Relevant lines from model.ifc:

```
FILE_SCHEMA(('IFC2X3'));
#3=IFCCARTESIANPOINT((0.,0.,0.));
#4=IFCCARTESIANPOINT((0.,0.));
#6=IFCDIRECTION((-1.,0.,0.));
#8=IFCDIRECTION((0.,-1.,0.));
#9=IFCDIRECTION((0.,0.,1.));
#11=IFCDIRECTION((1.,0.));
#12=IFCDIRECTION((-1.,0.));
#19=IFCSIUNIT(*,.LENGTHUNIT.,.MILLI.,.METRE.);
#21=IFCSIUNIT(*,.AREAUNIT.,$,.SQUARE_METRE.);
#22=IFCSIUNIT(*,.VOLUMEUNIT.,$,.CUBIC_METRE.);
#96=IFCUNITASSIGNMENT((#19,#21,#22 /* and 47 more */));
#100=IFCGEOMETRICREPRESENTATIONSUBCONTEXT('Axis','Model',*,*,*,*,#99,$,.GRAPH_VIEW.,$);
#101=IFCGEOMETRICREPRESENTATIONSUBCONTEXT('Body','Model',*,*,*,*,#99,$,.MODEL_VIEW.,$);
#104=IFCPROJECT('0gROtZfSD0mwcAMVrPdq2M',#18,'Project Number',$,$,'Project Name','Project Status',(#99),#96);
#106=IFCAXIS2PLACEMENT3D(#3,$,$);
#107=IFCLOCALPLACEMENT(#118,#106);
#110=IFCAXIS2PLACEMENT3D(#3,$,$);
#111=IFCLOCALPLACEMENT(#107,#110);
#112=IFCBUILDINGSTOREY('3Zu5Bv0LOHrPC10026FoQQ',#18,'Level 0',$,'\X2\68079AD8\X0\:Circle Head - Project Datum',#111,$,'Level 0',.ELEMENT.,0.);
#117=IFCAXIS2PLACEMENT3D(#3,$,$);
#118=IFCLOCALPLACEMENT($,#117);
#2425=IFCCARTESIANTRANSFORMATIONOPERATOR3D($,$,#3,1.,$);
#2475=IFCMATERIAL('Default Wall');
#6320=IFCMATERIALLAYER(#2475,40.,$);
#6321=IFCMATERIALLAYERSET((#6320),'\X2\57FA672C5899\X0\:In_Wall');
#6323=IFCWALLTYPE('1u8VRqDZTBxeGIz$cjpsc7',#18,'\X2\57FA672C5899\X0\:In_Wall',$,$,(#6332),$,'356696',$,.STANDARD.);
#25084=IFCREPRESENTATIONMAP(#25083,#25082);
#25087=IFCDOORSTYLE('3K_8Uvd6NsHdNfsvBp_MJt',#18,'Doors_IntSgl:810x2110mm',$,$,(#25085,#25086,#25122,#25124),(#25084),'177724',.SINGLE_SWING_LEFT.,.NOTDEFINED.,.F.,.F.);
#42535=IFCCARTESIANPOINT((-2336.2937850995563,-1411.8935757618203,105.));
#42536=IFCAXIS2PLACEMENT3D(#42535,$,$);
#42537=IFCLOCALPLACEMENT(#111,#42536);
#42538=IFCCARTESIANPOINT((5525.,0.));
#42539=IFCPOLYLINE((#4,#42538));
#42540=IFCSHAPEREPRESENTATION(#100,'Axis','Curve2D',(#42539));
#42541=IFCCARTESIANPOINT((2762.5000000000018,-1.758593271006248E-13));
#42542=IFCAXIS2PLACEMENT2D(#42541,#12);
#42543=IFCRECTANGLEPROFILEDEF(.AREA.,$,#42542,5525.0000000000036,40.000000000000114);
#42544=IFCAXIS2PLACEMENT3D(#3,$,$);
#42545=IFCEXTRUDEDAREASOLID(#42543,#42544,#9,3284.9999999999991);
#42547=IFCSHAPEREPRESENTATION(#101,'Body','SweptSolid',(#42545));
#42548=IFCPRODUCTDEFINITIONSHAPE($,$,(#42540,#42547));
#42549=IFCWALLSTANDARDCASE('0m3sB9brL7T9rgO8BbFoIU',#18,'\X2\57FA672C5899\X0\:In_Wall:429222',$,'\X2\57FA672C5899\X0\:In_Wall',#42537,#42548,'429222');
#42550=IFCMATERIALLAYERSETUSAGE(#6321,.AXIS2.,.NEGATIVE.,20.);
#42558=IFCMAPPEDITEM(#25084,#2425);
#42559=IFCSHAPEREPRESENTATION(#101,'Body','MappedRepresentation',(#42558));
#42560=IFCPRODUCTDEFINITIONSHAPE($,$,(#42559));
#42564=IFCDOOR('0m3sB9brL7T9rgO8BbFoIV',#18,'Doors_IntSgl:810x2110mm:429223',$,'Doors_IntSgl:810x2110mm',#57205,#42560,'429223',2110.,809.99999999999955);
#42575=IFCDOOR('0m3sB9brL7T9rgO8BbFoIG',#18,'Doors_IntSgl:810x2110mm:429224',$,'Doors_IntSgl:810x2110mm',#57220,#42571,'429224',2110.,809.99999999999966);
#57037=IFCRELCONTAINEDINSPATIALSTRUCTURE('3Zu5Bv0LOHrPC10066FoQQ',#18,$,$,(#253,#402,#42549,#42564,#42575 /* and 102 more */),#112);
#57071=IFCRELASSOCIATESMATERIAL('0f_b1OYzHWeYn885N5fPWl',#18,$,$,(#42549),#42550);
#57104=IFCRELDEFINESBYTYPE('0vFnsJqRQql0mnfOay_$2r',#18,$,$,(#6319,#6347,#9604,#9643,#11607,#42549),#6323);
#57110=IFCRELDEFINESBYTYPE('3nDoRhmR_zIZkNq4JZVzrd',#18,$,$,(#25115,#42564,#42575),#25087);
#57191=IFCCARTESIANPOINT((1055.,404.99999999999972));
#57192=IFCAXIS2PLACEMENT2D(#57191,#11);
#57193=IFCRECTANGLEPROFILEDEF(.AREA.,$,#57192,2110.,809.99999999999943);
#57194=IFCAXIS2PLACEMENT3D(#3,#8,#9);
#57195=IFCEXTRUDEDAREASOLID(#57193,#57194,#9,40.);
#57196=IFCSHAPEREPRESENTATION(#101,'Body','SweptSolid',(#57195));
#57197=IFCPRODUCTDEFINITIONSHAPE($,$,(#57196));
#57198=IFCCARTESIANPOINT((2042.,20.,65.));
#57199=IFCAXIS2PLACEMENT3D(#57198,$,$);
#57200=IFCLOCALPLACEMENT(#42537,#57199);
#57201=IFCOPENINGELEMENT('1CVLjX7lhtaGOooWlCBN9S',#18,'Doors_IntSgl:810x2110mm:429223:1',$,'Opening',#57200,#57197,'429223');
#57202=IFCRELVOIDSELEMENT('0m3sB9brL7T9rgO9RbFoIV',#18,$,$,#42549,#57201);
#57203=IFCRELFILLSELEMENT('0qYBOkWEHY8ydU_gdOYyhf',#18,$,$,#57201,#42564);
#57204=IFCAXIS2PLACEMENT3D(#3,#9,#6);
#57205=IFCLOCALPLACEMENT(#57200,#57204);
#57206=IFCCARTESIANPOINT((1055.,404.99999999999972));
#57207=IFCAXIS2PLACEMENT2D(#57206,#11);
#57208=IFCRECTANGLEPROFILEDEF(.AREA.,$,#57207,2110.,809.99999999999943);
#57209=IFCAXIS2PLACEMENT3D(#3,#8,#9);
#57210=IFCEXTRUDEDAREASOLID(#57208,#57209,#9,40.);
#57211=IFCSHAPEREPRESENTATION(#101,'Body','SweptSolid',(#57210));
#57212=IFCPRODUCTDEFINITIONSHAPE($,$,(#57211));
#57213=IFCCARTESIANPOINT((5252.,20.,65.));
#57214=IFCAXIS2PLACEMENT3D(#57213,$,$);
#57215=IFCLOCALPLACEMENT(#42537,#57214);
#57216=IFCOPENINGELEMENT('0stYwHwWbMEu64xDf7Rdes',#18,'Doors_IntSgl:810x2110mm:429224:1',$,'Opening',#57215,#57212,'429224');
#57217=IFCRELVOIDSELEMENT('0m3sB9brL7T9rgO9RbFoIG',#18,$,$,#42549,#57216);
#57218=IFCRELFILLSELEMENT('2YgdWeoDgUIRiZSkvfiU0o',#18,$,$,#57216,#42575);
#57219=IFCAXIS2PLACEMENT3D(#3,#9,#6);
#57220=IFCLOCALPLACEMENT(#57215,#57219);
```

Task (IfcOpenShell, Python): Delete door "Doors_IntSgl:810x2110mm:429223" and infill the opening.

```python
import ifcopenshell
import ifcopenshell.api.feature
import ifcopenshell.api.root
import ifcopenshell.geom
import ifcopenshell.util.shape

model = ifcopenshell.open("model.ifc")
settings = ifcopenshell.geom.settings()


def volume(element):
    """Net volume in cubic metres, openings subtracted."""
    shape = ifcopenshell.geom.create_shape(settings, element)
    return ifcopenshell.util.shape.get_volume(shape.geometry)


door = model.by_guid("0m3sB9brL7T9rgO8BbFoIV")
opening = door.FillsVoids[0].RelatingOpeningElement
wall = opening.VoidsElements[0].RelatingBuildingElement
before = volume(wall)

ifcopenshell.api.root.remove_product(model, product=door)
ifcopenshell.api.feature.remove_feature(model, feature=opening)

after = volume(wall)

print(f"wall volume {before:.3f} -> {after:.3f} m3")

model.write("model_updated.ifc")
```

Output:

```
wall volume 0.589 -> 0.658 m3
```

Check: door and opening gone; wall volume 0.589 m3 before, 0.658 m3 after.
